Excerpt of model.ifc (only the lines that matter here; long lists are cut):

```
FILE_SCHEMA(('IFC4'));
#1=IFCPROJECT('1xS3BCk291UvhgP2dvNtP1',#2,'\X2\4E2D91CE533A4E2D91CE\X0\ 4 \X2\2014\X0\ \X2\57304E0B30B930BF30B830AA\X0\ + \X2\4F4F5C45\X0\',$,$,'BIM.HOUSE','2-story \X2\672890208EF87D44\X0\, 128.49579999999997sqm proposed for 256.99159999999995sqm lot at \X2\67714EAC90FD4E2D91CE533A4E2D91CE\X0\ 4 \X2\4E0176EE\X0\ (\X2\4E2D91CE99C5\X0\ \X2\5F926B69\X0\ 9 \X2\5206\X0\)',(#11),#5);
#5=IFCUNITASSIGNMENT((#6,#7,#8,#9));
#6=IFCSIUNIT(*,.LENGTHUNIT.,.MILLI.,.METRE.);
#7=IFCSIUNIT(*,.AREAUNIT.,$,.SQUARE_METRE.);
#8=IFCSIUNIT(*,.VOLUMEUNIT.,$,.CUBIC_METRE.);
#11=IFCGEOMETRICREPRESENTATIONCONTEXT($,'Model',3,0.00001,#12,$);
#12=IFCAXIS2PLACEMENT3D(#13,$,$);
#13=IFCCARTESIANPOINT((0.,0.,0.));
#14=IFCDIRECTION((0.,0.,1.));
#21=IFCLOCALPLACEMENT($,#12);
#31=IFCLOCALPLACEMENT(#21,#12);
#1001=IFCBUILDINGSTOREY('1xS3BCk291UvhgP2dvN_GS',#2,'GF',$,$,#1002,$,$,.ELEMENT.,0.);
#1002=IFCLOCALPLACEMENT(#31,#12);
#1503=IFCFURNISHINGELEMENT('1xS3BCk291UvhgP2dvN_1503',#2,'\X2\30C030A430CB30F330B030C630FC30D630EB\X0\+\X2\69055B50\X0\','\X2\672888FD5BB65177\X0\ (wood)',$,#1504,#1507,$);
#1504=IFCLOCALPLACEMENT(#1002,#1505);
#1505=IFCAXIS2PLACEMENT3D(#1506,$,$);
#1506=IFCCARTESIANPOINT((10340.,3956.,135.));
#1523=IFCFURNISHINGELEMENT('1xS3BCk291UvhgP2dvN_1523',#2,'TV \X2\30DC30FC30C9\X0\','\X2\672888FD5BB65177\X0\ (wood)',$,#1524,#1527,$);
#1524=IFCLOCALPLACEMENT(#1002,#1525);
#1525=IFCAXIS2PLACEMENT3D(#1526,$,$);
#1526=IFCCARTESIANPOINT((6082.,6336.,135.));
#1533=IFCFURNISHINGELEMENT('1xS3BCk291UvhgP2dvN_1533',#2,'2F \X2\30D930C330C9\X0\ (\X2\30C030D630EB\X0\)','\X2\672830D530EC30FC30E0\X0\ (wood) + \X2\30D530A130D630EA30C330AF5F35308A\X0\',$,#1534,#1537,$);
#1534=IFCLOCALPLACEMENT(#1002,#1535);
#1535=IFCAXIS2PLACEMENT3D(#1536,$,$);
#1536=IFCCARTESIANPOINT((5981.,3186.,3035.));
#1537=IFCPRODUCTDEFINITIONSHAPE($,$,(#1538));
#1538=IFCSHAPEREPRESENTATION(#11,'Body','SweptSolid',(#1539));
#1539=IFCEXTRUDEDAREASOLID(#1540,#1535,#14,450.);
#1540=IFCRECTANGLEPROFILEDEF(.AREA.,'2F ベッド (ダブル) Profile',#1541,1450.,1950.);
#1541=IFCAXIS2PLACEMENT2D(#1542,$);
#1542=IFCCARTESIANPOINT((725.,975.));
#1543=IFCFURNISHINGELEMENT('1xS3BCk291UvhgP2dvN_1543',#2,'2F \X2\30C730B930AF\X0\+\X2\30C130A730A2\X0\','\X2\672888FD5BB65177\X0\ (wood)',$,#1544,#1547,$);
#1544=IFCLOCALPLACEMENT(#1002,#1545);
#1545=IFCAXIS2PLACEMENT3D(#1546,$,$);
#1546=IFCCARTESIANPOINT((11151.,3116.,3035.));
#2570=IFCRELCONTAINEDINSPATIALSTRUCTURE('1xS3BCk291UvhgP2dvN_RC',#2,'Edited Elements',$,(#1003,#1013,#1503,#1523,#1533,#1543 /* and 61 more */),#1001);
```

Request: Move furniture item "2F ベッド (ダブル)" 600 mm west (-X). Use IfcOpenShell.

```python
import ifcopenshell
import ifcopenshell.api.geometry
import ifcopenshell.util.placement
import ifcopenshell.util.unit

model = ifcopenshell.open("model.ifc")
unit_scale = ifcopenshell.util.unit.calculate_unit_scale(model)

item = model.by_guid("1xS3BCk291UvhgP2dvN_1533")
matrix = ifcopenshell.util.placement.get_local_placement(item.ObjectPlacement)
matrix[0, 3] -= 0.6 / unit_scale
ifcopenshell.api.geometry.edit_object_placement(model, product=item, matrix=matrix, is_si=False)

print(ifcopenshell.util.placement.get_local_placement(item.ObjectPlacement).round(3) + 0.0)

model.write("model-out.ifc")
```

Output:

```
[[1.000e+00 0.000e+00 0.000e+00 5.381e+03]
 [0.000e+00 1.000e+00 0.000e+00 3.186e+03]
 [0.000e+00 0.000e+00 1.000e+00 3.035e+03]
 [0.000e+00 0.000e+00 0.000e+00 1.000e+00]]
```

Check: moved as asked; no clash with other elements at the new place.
